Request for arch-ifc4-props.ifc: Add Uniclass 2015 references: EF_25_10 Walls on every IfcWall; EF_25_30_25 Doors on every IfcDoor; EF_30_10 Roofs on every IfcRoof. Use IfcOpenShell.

First a look at what the model holds.

```python
import ifcopenshell

model = ifcopenshell.open("arch-ifc4-props.ifc")
print(model.schema)
print("classifications:", [c.Name for c in model.by_type("IfcClassification")])
for ifc_class in ("IfcDoor", "IfcRoof", "IfcStair", "IfcWall", "IfcWindow"):
    print(ifc_class, len(model.by_type(ifc_class)))
```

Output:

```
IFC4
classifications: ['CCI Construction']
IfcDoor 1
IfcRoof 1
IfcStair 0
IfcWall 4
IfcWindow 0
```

```python
import ifcopenshell
import ifcopenshell.api.classification

model = ifcopenshell.open("arch-ifc4-props.ifc")

system = ifcopenshell.api.classification.add_classification(model, classification="Uniclass 2015")

codes = {
    "IfcWall": ("EF_25_10", "Walls"),
    "IfcDoor": ("EF_25_30_25", "Doors"),
    "IfcRoof": ("EF_30_10", "Roofs"),
}
for ifc_class, (code, name) in codes.items():
    products = model.by_type(ifc_class)
    ifcopenshell.api.classification.add_reference(
        model, products=products, classification=system, identification=code, name=name
    )
    print(code, len(products))

model.write("arch-ifc4-props_updated.ifc")
```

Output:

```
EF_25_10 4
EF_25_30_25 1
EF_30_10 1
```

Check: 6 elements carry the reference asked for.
